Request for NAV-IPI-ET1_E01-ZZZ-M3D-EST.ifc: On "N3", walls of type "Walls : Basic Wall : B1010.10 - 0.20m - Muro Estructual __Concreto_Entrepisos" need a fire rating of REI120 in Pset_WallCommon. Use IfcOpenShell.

First a look at what the model holds.

```python
import ifcopenshell
import ifcopenshell.util.element

model = ifcopenshell.open("NAV-IPI-ET1_E01-ZZZ-M3D-EST.ifc")
print(model.schema)
storey = next(s for s in model.by_type("IfcBuildingStorey") if s.Name == "N3")
walls = [e for e in ifcopenshell.util.element.get_decomposition(storey) if e.is_a("IfcWall")]
seen = {}
for e in walls:
    element_type = ifcopenshell.util.element.get_type(e)
    key = (element_type.Name if element_type != e and element_type else None, ifcopenshell.util.element.get_pset(e, "Pset_WallCommon", "FireRating"))
    seen[key] = seen.get(key, 0) + 1
for (name, value), count in sorted(seen.items(), key=str):
    print(count, "x", name, "|", value)
```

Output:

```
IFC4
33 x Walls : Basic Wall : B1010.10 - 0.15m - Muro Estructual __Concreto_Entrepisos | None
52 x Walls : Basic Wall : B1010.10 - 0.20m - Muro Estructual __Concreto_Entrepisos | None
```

```python
import ifcopenshell
import ifcopenshell.api.pset
import ifcopenshell.util.element

model = ifcopenshell.open("NAV-IPI-ET1_E01-ZZZ-M3D-EST.ifc")

storey = next(s for s in model.by_type("IfcBuildingStorey") if s.Name == "N3")
walls = [e for e in ifcopenshell.util.element.get_decomposition(storey) if e.is_a("IfcWall")]

count = 0
for e in walls:
    element_type = ifcopenshell.util.element.get_type(e)
    if element_type in (None, e) or element_type.Name != "Walls : Basic Wall : B1010.10 - 0.20m - Muro Estructual __Concreto_Entrepisos":
        continue
    # add_pset returns the element's existing set when there is one.
    pset = ifcopenshell.api.pset.add_pset(model, product=e, name="Pset_WallCommon")
    ifcopenshell.api.pset.edit_pset(model, pset=pset, properties={"FireRating": "REI120"})
    count += 1

print(count, "walls updated")

model.write("NAV-IPI-ET1_E01-ZZZ-M3D-EST_updated.ifc")
```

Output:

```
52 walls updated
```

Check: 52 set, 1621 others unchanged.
